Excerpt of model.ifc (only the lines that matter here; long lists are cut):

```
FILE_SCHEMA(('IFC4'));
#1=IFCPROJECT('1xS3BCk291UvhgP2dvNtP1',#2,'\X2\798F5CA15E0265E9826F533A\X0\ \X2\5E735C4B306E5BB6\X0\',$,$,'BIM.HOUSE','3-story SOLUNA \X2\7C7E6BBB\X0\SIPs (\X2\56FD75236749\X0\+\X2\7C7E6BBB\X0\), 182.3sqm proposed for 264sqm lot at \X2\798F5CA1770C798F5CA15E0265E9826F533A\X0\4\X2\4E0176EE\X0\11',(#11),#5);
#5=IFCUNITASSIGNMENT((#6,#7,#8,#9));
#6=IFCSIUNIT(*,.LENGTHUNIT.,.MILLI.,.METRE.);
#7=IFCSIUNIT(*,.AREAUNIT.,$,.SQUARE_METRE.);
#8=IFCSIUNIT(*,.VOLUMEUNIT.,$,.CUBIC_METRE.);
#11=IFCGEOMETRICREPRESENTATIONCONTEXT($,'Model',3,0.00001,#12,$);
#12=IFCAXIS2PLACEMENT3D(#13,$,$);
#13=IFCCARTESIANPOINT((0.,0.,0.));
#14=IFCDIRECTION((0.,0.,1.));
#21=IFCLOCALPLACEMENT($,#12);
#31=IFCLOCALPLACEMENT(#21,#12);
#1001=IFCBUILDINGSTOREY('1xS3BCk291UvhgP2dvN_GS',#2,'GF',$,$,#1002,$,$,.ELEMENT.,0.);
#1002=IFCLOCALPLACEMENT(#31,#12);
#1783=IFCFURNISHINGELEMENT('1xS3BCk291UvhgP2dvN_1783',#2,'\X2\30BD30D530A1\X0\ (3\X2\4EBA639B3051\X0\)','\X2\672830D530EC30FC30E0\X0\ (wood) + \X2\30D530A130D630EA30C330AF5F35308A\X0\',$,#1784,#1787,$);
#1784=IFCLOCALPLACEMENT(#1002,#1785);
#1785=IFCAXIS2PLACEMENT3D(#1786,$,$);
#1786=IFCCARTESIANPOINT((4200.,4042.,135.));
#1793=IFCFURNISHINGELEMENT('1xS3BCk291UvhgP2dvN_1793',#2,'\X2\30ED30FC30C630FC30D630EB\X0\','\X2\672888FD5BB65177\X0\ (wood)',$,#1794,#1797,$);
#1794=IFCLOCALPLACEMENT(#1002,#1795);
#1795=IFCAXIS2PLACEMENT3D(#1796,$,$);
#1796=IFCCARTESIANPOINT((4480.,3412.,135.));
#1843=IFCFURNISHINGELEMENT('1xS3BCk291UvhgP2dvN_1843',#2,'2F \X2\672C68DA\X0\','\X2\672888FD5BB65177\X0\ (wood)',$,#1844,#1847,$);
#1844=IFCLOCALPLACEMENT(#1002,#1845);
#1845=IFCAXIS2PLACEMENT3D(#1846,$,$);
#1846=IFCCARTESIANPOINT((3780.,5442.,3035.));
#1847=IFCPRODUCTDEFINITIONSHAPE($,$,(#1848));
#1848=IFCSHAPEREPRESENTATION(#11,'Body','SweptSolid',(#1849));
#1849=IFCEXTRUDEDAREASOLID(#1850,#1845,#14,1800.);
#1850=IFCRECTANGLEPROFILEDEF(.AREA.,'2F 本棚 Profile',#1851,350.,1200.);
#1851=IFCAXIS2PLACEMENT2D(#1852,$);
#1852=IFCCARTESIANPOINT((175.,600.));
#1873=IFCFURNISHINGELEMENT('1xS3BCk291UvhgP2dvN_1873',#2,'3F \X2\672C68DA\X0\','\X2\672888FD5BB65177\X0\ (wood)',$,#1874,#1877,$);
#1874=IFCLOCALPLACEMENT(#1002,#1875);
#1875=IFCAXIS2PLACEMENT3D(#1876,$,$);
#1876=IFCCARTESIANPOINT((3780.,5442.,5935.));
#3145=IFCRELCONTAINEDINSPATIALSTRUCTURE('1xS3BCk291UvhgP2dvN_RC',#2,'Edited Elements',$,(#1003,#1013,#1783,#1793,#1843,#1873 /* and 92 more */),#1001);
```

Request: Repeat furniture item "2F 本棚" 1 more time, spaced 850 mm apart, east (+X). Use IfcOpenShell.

```python
import numpy as np
import ifcopenshell
import ifcopenshell.api.geometry
import ifcopenshell.api.root
import ifcopenshell.util.element
import ifcopenshell.util.placement
import ifcopenshell.util.unit

model = ifcopenshell.open("model.ifc")
unit_scale = ifcopenshell.util.unit.calculate_unit_scale(model)


def reuse_history(source, copy):
    """copy_class also copies each property set's owner history, people and application; keep the originals."""
    for rel in copy.IsDefinedBy:
        if rel.is_a("IfcRelDefinesByProperties") and (history := rel.RelatingPropertyDefinition.OwnerHistory):
            rel.RelatingPropertyDefinition.OwnerHistory = source.OwnerHistory
            ifcopenshell.util.element.remove_deep2(model, history)


source = model.by_guid("1xS3BCk291UvhgP2dvN_1843")
base = ifcopenshell.util.placement.get_local_placement(source.ObjectPlacement)
step = np.array([1.0, 0.0, 0.0]) * 0.85 / unit_scale

for i in range(1, 2):
    copy = ifcopenshell.api.root.copy_class(model, product=source)
    copy.Representation = ifcopenshell.util.element.copy_deep(
        model, source.Representation, exclude=["IfcGeometricRepresentationContext", "IfcRepresentationMap"]
    )
    reuse_history(source, copy)
    matrix = base.copy()
    matrix[:3, 3] += i * step
    print("added at", matrix[:3, 3].round(3) + 0.0)
    ifcopenshell.api.geometry.edit_object_placement(model, product=copy, matrix=matrix, is_si=False)

model.write("model_edited.ifc")
```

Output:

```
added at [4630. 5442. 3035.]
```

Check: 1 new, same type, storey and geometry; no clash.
